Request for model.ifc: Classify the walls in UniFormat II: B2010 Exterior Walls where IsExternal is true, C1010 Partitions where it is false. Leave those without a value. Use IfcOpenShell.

First a look at what the model holds.

```python
import ifcopenshell
import ifcopenshell.util.element

model = ifcopenshell.open("model.ifc")
print(model.schema)
print("classifications:", [c.Name for c in model.by_type("IfcClassification")])
values = [ifcopenshell.util.element.get_pset(e, "Pset_WallCommon", "IsExternal") for e in model.by_type("IfcWall")]
for value in (True, False, None):
    print("IsExternal", value, values.count(value))
```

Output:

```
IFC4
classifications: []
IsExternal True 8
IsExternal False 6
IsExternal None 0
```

```python
import ifcopenshell
import ifcopenshell.api.classification
import ifcopenshell.util.element

model = ifcopenshell.open("model.ifc")

system = ifcopenshell.api.classification.add_classification(model, classification="UniFormat II")

walls = model.by_type("IfcWall")
external = {e: ifcopenshell.util.element.get_pset(e, "Pset_WallCommon", "IsExternal") for e in walls}
for flag, code, name in ((True, "B2010", "Exterior Walls"), (False, "C1010", "Partitions")):
    products = [e for e in walls if external[e] is flag]
    ifcopenshell.api.classification.add_reference(
        model, products=products, classification=system, identification=code, name=name
    )
    print(code, len(products))

model.write("model_edited.ifc")
```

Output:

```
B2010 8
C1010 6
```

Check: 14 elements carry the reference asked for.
